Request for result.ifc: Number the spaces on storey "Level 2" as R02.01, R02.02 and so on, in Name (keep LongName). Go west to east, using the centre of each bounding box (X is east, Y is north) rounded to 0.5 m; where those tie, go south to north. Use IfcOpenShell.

First a look at what the model holds.

```python
import ifcopenshell
import ifcopenshell.util.element
import ifcopenshell.util.placement

model = ifcopenshell.open("result.ifc")
print(model.schema)
storey = next(s for s in model.by_type("IfcBuildingStorey") if s.Name == "Level 2")
spaces = [e for e in ifcopenshell.util.element.get_decomposition(storey) if e.is_a("IfcSpace")]
for e in sorted(spaces, key=lambda e: e.id()):
    origin = ifcopenshell.util.placement.get_local_placement(e.ObjectPlacement)[:3, 3]
    print(e.id(), e.Name, e.LongName, origin.round(2) + 0.0, sep=" | ")
```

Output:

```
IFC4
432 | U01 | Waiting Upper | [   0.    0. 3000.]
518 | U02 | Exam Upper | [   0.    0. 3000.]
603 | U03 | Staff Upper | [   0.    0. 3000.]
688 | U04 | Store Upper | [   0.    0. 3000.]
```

```python
import ifcopenshell
import ifcopenshell.geom
import ifcopenshell.util.element
import ifcopenshell.util.shape

model = ifcopenshell.open("result.ifc")
settings = ifcopenshell.geom.settings()
settings.set("use-world-coords", True)


def centre(element):
    shape = ifcopenshell.geom.create_shape(settings, element)
    return ifcopenshell.util.shape.get_bbox_centroid(shape.geometry)


storey = next(s for s in model.by_type("IfcBuildingStorey") if s.Name == "Level 2")
spaces = [e for e in ifcopenshell.util.element.get_decomposition(storey) if e.is_a("IfcSpace")]

# Insertion points can sit at a corner or the storey origin, so sort by the geometry (in metres).
centres = {e: centre(e) for e in spaces}
spaces.sort(key=lambda e: (round(centres[e][0] / 0.5), centres[e][1]))

for i, e in enumerate(spaces, start=1):
    number = f"R02.{i:02d}"
    e.Name = number
    print(e.id(), number)

model.write("result_updated.ifc")
```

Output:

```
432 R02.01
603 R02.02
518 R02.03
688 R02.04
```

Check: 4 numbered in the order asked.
